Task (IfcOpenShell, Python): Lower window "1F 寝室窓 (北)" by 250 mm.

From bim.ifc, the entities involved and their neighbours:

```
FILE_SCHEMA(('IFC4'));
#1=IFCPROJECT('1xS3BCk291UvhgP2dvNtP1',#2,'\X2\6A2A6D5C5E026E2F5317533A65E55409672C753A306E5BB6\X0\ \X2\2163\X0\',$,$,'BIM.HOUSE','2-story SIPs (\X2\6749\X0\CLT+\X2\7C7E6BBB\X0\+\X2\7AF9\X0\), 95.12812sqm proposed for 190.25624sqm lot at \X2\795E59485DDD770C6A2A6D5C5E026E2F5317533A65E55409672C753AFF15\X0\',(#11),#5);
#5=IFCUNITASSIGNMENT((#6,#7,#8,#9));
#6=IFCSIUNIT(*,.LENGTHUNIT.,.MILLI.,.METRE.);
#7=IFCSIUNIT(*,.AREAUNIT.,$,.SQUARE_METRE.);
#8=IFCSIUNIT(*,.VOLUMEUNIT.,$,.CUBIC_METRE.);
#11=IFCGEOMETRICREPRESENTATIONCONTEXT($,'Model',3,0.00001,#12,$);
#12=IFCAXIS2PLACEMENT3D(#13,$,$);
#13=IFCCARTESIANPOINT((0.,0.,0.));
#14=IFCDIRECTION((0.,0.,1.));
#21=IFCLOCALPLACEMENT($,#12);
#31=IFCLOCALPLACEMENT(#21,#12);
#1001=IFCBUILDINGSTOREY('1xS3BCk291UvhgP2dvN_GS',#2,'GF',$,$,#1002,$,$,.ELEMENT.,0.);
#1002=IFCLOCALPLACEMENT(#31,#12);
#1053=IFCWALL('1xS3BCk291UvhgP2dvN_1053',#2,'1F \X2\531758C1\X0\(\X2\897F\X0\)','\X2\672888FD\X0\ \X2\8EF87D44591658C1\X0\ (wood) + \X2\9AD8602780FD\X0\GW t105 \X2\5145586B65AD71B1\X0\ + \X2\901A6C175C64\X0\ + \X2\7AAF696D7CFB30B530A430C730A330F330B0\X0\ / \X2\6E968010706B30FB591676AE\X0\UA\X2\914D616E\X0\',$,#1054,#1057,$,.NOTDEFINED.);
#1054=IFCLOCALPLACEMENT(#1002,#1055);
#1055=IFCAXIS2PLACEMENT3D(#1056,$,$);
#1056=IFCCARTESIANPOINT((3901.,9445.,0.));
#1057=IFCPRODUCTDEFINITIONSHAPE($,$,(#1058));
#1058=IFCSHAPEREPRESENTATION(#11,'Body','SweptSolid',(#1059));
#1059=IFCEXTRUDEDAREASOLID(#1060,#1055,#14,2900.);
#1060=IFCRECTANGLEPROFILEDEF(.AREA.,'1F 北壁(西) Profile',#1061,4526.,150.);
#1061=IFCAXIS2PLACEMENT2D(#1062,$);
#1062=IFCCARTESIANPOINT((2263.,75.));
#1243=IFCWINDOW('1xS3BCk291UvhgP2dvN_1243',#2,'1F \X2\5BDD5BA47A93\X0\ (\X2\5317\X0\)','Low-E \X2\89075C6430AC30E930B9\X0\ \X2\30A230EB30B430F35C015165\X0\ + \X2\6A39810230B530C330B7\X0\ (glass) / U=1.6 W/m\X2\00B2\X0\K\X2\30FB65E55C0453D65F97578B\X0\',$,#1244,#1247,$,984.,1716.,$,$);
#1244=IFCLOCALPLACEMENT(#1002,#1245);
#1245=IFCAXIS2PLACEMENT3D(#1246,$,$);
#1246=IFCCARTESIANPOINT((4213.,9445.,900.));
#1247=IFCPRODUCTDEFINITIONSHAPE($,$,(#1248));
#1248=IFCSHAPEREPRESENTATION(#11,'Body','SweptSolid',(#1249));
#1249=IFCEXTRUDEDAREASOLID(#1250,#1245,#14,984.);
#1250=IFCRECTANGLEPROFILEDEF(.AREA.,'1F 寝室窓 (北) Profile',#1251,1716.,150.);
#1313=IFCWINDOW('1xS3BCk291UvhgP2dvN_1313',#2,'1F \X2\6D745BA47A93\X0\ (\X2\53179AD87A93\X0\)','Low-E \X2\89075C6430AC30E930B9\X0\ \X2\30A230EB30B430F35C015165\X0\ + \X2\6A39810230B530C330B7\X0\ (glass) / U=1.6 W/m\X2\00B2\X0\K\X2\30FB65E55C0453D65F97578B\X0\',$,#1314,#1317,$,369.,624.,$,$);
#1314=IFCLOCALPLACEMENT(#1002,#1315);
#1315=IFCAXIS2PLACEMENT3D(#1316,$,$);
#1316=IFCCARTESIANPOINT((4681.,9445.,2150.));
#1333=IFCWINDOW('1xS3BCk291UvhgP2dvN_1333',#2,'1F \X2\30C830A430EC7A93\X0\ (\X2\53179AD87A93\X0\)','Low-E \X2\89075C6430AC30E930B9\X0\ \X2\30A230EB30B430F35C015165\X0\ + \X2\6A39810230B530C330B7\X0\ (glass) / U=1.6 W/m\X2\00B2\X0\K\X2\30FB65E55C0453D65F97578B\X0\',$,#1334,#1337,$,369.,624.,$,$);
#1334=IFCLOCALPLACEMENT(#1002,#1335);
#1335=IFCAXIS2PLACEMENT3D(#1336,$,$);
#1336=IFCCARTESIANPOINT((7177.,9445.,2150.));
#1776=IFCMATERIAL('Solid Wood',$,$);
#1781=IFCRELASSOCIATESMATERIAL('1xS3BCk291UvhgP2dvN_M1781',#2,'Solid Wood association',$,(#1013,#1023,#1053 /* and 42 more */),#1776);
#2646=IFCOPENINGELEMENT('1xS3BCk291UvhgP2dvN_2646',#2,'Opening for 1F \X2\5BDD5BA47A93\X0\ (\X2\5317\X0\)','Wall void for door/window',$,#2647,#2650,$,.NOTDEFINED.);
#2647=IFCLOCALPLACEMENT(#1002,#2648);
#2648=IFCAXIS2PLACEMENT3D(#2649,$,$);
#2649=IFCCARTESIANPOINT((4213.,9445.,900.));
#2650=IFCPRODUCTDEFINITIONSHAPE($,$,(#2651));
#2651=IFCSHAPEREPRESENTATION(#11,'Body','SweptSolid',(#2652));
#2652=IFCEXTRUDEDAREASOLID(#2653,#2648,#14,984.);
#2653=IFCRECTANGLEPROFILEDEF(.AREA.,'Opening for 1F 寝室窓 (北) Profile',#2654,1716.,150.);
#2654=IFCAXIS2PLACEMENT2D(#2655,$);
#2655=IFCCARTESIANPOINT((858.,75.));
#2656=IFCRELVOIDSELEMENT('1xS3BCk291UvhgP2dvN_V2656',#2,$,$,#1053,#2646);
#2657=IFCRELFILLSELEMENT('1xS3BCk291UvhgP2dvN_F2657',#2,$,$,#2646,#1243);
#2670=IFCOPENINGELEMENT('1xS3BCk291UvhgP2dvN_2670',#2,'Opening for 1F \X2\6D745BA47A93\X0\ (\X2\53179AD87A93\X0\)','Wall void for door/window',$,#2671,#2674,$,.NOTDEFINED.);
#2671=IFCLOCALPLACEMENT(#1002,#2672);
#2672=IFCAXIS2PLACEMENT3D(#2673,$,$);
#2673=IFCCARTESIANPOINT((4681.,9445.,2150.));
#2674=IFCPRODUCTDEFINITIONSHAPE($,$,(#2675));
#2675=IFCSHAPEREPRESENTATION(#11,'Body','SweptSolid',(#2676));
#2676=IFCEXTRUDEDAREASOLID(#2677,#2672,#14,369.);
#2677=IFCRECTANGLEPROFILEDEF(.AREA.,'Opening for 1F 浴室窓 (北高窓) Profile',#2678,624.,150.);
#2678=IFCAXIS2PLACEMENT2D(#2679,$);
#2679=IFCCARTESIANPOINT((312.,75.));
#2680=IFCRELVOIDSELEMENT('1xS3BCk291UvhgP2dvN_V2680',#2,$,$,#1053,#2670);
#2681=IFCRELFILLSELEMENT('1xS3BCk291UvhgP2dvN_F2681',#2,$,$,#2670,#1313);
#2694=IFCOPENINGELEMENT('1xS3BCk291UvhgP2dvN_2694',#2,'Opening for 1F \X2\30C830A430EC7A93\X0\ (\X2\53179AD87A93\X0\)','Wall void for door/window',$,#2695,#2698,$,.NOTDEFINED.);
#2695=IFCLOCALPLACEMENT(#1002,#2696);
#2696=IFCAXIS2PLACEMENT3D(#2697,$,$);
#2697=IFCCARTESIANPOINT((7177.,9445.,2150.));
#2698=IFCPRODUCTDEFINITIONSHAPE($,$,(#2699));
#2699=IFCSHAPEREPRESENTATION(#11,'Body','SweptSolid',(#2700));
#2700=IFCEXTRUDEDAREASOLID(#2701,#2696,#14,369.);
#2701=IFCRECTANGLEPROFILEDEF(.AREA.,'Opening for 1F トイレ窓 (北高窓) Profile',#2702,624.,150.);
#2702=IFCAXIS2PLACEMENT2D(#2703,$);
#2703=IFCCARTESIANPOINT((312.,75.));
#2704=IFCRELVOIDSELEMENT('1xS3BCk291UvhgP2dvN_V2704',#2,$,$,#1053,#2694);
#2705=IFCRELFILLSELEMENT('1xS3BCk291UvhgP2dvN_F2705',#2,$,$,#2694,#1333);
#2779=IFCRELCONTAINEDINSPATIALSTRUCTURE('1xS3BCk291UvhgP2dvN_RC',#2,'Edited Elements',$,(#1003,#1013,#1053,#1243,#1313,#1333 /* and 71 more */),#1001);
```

```python
import numpy as np
import ifcopenshell
import ifcopenshell.api.geometry
import ifcopenshell.util.placement
import ifcopenshell.util.unit

model = ifcopenshell.open("bim.ifc")
unit_scale = ifcopenshell.util.unit.calculate_unit_scale(model)

window = model.by_id(1243)
opening = window.FillsVoids[0].RelatingOpeningElement
dz = -0.25 / unit_scale

shift = np.array([0.0, 0.0, dz])
# The window is not placed relative to its opening, so move both.
for product in (opening, window):
    matrix = ifcopenshell.util.placement.get_local_placement(product.ObjectPlacement)
    matrix[:3, 3] += shift
    ifcopenshell.api.geometry.edit_object_placement(model, product=product, matrix=matrix, is_si=False)

print(f"moved by {dz * unit_scale:+.3f} m")

model.write("bim_edited.ifc")
```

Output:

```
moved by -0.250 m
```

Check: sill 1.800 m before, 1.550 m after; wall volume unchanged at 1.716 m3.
